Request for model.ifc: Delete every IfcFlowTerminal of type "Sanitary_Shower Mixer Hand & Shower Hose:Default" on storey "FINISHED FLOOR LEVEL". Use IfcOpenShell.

First a look at what the model holds.

```python
import ifcopenshell
import ifcopenshell.util.element

model = ifcopenshell.open("model.ifc")
print(model.schema)
storey = next(s for s in model.by_type("IfcBuildingStorey") if s.Name == "FINISHED FLOOR LEVEL")
terminals = [e for e in ifcopenshell.util.element.get_decomposition(storey) if e.is_a("IfcFlowTerminal")]
seen = {}
for e in terminals:
    element_type = ifcopenshell.util.element.get_type(e)
    name = element_type.Name if element_type not in (None, e) else None
    seen[name] = seen.get(name, 0) + 1
for name, count in sorted(seen.items(), key=str):
    print(count, "x", name)
```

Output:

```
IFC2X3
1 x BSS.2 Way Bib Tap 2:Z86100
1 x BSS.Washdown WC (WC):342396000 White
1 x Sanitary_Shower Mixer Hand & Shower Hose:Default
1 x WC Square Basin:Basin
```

```python
import ifcopenshell
import ifcopenshell.api.root
import ifcopenshell.util.element

model = ifcopenshell.open("model.ifc")

storey = next(s for s in model.by_type("IfcBuildingStorey") if s.Name == "FINISHED FLOOR LEVEL")
terminals = [e for e in ifcopenshell.util.element.get_decomposition(storey) if e.is_a("IfcFlowTerminal")]
targets = [e for e in terminals if (t := ifcopenshell.util.element.get_type(e)) not in (None, e) and t.Name == "Sanitary_Shower Mixer Hand & Shower Hose:Default"]

for e in targets:
    ifcopenshell.api.root.remove_product(model, product=e)
print(len(targets), "removed")

model.write("model_rev.ifc")
```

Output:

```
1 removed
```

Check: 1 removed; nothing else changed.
